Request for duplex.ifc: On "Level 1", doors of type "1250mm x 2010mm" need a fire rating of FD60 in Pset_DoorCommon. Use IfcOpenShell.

First a look at what the model holds.

```python
import ifcopenshell
import ifcopenshell.util.element

model = ifcopenshell.open("duplex.ifc")
print(model.schema)
storey = next(s for s in model.by_type("IfcBuildingStorey") if s.Name == "Level 1")
doors = [e for e in ifcopenshell.util.element.get_decomposition(storey) if e.is_a("IfcDoor")]
seen = {}
for e in doors:
    element_type = ifcopenshell.util.element.get_type(e)
    key = (element_type.Name if element_type != e and element_type else None, ifcopenshell.util.element.get_pset(e, "Pset_DoorCommon", "FireRating"))
    seen[key] = seen.get(key, 0) + 1
for (name, value), count in sorted(seen.items(), key=str):
    print(count, "x", name, "|", value)
```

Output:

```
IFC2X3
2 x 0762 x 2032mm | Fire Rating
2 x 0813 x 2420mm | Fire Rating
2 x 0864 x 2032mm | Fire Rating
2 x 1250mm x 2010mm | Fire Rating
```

```python
import ifcopenshell
import ifcopenshell.api.pset
import ifcopenshell.util.element

model = ifcopenshell.open("duplex.ifc")

storey = next(s for s in model.by_type("IfcBuildingStorey") if s.Name == "Level 1")
doors = [e for e in ifcopenshell.util.element.get_decomposition(storey) if e.is_a("IfcDoor")]

count = 0
for e in doors:
    element_type = ifcopenshell.util.element.get_type(e)
    if element_type in (None, e) or element_type.Name != "1250mm x 2010mm":
        continue
    # add_pset returns the element's existing set when there is one.
    pset = ifcopenshell.api.pset.add_pset(model, product=e, name="Pset_DoorCommon")
    ifcopenshell.api.pset.edit_pset(model, pset=pset, properties={"FireRating": "FD60"})
    count += 1

print(count, "doors updated")

model.write("duplex_updated.ifc")
```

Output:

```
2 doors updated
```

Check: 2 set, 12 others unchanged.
